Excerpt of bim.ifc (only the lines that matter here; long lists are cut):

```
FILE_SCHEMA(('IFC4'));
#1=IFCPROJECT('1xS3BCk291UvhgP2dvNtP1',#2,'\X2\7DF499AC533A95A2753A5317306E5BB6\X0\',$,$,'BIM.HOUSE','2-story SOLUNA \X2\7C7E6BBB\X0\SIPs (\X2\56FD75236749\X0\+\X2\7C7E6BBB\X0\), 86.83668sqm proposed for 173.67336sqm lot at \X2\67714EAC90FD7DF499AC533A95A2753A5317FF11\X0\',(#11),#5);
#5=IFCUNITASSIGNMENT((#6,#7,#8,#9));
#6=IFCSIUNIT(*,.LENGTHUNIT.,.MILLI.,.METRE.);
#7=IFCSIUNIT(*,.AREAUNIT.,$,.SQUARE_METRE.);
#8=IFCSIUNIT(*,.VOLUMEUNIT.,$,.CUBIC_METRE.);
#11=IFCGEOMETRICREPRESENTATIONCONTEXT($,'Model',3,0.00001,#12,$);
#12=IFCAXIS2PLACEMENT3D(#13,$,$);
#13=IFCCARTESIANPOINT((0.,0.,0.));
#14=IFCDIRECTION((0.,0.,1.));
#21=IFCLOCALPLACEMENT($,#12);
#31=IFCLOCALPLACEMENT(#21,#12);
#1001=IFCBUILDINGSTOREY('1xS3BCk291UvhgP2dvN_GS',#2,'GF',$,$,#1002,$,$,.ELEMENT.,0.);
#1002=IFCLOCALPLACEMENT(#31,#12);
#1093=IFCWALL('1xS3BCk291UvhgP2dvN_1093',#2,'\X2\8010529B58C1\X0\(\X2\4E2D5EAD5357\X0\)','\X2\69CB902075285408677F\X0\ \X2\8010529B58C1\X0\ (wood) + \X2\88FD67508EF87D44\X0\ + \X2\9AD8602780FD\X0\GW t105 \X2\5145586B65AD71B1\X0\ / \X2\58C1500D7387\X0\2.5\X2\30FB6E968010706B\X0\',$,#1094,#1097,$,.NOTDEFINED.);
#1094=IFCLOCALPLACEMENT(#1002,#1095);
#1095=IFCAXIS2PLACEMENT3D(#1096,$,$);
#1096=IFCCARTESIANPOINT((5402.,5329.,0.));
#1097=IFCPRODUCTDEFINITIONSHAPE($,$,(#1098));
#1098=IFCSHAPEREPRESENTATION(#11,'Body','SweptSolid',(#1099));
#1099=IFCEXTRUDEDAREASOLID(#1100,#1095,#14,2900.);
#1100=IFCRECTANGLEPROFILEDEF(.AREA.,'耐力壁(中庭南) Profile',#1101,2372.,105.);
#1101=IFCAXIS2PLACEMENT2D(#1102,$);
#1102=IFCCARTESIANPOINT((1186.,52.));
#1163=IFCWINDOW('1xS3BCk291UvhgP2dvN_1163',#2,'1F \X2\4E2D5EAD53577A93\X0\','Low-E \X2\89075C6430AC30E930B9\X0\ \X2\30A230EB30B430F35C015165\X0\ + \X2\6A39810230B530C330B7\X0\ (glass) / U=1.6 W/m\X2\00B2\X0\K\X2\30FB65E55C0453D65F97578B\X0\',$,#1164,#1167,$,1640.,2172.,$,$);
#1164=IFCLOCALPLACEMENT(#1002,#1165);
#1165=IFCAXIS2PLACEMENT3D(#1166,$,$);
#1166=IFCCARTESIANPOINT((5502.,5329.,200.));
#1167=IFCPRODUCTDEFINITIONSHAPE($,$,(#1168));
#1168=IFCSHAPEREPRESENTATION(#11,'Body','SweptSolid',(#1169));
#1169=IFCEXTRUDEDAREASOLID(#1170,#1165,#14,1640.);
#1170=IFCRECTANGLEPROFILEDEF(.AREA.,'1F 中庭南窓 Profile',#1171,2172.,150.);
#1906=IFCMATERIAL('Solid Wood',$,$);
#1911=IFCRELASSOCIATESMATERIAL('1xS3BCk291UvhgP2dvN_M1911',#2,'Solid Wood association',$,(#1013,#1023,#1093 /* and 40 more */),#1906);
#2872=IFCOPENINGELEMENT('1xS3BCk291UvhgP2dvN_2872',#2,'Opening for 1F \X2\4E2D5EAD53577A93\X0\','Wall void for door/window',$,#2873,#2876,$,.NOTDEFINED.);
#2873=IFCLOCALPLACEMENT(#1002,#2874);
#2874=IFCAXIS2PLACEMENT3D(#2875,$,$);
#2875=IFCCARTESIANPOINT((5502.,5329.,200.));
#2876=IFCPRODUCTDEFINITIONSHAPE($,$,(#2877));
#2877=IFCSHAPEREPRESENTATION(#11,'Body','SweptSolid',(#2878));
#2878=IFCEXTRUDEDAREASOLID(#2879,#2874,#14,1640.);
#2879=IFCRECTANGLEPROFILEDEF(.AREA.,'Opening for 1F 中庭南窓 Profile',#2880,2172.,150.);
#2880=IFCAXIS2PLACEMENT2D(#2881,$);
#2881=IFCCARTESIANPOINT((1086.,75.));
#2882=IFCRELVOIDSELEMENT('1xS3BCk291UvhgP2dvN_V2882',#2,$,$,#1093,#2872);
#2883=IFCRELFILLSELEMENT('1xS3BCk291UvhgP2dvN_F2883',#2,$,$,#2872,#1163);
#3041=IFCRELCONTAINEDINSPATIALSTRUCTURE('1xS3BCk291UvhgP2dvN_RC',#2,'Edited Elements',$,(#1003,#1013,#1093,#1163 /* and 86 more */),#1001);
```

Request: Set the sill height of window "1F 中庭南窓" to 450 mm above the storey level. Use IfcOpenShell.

```python
import numpy as np
import ifcopenshell
import ifcopenshell.api.geometry
import ifcopenshell.geom
import ifcopenshell.util.element
import ifcopenshell.util.placement
import ifcopenshell.util.shape
import ifcopenshell.util.unit

model = ifcopenshell.open("bim.ifc")
unit_scale = ifcopenshell.util.unit.calculate_unit_scale(model)

window = model.by_guid("1xS3BCk291UvhgP2dvN_1163")
opening = window.FillsVoids[0].RelatingOpeningElement
storey = ifcopenshell.util.element.get_container(window, ifc_class="IfcBuildingStorey")
level = ifcopenshell.util.placement.get_local_placement(storey.ObjectPlacement)[2, 3]

# The opening's origin need not be at the sill, so measure its lowest point.
shape = ifcopenshell.geom.create_shape(ifcopenshell.geom.settings(), opening)
bottom = ifcopenshell.util.shape.get_shape_bottom_elevation(shape, shape.geometry) / unit_scale
dz = level + 0.45 / unit_scale - bottom

shift = np.array([0.0, 0.0, dz])
# The window is not placed relative to its opening, so move both.
for product in (opening, window):
    matrix = ifcopenshell.util.placement.get_local_placement(product.ObjectPlacement)
    matrix[:3, 3] += shift
    ifcopenshell.api.geometry.edit_object_placement(model, product=product, matrix=matrix, is_si=False)

print(f"moved by {dz * unit_scale:+.3f} m")

model.write("bim_updated.ifc")
```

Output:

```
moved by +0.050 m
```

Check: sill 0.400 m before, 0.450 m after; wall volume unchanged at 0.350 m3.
